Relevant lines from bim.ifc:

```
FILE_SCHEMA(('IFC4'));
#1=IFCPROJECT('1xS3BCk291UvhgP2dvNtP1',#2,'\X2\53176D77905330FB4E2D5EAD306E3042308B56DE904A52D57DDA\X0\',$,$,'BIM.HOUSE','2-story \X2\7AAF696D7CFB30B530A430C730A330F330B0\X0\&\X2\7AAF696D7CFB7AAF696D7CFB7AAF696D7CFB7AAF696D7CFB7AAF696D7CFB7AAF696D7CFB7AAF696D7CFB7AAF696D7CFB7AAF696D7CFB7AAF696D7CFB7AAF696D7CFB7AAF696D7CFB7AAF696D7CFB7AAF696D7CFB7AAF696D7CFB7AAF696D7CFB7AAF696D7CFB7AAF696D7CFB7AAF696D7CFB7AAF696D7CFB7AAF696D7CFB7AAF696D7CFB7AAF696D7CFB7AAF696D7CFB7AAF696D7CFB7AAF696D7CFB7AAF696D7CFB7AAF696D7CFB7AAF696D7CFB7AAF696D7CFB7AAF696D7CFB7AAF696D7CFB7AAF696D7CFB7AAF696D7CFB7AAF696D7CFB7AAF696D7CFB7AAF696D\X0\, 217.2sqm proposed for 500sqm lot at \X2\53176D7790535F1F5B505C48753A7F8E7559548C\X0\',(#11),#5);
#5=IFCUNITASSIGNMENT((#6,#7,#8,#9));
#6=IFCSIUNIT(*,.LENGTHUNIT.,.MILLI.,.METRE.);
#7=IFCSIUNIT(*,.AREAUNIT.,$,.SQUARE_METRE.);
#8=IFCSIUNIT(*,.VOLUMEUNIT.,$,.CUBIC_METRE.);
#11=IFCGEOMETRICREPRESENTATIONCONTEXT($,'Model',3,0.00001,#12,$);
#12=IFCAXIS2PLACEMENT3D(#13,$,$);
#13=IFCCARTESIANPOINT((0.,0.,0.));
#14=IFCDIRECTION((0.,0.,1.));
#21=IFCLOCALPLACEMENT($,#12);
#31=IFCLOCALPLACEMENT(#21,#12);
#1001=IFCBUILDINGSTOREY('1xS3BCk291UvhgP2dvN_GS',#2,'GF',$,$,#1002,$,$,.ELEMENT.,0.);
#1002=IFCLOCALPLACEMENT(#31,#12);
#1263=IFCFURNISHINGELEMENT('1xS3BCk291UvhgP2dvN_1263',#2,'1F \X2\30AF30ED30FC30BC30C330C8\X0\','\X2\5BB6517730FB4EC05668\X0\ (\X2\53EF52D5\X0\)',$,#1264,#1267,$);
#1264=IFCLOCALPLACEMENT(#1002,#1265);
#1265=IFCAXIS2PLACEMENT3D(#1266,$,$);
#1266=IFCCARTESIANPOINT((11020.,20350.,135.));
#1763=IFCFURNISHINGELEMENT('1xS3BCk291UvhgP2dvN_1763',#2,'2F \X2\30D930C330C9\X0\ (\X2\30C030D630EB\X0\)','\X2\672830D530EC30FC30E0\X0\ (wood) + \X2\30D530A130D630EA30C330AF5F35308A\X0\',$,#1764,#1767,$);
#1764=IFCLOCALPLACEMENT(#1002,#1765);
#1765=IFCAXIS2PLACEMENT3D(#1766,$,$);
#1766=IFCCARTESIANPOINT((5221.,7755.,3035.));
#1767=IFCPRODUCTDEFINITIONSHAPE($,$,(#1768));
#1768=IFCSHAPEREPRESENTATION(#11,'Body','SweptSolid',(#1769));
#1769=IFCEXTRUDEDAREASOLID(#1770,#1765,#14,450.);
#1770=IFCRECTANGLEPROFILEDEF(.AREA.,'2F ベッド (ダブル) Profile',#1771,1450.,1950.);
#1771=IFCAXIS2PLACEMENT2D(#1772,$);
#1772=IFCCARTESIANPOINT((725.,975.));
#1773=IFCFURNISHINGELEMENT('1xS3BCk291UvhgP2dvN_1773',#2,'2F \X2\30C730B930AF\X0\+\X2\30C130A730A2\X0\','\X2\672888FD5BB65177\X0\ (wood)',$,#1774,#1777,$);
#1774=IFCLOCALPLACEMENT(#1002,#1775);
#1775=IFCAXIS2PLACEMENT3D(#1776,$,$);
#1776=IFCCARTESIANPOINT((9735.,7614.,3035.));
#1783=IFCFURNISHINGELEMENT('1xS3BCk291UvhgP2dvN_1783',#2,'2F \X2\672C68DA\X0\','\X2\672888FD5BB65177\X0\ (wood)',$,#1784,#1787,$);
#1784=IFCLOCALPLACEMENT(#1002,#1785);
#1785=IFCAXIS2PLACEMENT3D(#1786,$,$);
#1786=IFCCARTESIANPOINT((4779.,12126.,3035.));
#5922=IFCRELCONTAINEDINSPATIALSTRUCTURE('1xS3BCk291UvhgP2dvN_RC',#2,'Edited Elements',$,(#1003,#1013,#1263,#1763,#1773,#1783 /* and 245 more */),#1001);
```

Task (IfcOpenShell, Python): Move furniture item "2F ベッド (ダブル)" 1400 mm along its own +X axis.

```python
import ifcopenshell
import ifcopenshell.api.geometry
import ifcopenshell.util.placement

model = ifcopenshell.open("bim.ifc")

item = model.by_guid("1xS3BCk291UvhgP2dvN_1763")
matrix = ifcopenshell.util.placement.get_local_placement(item.ObjectPlacement)
matrix[:3, 3] += matrix[:3, 0] * 1400.0
ifcopenshell.api.geometry.edit_object_placement(model, product=item, matrix=matrix, is_si=False)

print(ifcopenshell.util.placement.get_local_placement(item.ObjectPlacement).round(3) + 0.0)

model.write("bim_updated.ifc")
```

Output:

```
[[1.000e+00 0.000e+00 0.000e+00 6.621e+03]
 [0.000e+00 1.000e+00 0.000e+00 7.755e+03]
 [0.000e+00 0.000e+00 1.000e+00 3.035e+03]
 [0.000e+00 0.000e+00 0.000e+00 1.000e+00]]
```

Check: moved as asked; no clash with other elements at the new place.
